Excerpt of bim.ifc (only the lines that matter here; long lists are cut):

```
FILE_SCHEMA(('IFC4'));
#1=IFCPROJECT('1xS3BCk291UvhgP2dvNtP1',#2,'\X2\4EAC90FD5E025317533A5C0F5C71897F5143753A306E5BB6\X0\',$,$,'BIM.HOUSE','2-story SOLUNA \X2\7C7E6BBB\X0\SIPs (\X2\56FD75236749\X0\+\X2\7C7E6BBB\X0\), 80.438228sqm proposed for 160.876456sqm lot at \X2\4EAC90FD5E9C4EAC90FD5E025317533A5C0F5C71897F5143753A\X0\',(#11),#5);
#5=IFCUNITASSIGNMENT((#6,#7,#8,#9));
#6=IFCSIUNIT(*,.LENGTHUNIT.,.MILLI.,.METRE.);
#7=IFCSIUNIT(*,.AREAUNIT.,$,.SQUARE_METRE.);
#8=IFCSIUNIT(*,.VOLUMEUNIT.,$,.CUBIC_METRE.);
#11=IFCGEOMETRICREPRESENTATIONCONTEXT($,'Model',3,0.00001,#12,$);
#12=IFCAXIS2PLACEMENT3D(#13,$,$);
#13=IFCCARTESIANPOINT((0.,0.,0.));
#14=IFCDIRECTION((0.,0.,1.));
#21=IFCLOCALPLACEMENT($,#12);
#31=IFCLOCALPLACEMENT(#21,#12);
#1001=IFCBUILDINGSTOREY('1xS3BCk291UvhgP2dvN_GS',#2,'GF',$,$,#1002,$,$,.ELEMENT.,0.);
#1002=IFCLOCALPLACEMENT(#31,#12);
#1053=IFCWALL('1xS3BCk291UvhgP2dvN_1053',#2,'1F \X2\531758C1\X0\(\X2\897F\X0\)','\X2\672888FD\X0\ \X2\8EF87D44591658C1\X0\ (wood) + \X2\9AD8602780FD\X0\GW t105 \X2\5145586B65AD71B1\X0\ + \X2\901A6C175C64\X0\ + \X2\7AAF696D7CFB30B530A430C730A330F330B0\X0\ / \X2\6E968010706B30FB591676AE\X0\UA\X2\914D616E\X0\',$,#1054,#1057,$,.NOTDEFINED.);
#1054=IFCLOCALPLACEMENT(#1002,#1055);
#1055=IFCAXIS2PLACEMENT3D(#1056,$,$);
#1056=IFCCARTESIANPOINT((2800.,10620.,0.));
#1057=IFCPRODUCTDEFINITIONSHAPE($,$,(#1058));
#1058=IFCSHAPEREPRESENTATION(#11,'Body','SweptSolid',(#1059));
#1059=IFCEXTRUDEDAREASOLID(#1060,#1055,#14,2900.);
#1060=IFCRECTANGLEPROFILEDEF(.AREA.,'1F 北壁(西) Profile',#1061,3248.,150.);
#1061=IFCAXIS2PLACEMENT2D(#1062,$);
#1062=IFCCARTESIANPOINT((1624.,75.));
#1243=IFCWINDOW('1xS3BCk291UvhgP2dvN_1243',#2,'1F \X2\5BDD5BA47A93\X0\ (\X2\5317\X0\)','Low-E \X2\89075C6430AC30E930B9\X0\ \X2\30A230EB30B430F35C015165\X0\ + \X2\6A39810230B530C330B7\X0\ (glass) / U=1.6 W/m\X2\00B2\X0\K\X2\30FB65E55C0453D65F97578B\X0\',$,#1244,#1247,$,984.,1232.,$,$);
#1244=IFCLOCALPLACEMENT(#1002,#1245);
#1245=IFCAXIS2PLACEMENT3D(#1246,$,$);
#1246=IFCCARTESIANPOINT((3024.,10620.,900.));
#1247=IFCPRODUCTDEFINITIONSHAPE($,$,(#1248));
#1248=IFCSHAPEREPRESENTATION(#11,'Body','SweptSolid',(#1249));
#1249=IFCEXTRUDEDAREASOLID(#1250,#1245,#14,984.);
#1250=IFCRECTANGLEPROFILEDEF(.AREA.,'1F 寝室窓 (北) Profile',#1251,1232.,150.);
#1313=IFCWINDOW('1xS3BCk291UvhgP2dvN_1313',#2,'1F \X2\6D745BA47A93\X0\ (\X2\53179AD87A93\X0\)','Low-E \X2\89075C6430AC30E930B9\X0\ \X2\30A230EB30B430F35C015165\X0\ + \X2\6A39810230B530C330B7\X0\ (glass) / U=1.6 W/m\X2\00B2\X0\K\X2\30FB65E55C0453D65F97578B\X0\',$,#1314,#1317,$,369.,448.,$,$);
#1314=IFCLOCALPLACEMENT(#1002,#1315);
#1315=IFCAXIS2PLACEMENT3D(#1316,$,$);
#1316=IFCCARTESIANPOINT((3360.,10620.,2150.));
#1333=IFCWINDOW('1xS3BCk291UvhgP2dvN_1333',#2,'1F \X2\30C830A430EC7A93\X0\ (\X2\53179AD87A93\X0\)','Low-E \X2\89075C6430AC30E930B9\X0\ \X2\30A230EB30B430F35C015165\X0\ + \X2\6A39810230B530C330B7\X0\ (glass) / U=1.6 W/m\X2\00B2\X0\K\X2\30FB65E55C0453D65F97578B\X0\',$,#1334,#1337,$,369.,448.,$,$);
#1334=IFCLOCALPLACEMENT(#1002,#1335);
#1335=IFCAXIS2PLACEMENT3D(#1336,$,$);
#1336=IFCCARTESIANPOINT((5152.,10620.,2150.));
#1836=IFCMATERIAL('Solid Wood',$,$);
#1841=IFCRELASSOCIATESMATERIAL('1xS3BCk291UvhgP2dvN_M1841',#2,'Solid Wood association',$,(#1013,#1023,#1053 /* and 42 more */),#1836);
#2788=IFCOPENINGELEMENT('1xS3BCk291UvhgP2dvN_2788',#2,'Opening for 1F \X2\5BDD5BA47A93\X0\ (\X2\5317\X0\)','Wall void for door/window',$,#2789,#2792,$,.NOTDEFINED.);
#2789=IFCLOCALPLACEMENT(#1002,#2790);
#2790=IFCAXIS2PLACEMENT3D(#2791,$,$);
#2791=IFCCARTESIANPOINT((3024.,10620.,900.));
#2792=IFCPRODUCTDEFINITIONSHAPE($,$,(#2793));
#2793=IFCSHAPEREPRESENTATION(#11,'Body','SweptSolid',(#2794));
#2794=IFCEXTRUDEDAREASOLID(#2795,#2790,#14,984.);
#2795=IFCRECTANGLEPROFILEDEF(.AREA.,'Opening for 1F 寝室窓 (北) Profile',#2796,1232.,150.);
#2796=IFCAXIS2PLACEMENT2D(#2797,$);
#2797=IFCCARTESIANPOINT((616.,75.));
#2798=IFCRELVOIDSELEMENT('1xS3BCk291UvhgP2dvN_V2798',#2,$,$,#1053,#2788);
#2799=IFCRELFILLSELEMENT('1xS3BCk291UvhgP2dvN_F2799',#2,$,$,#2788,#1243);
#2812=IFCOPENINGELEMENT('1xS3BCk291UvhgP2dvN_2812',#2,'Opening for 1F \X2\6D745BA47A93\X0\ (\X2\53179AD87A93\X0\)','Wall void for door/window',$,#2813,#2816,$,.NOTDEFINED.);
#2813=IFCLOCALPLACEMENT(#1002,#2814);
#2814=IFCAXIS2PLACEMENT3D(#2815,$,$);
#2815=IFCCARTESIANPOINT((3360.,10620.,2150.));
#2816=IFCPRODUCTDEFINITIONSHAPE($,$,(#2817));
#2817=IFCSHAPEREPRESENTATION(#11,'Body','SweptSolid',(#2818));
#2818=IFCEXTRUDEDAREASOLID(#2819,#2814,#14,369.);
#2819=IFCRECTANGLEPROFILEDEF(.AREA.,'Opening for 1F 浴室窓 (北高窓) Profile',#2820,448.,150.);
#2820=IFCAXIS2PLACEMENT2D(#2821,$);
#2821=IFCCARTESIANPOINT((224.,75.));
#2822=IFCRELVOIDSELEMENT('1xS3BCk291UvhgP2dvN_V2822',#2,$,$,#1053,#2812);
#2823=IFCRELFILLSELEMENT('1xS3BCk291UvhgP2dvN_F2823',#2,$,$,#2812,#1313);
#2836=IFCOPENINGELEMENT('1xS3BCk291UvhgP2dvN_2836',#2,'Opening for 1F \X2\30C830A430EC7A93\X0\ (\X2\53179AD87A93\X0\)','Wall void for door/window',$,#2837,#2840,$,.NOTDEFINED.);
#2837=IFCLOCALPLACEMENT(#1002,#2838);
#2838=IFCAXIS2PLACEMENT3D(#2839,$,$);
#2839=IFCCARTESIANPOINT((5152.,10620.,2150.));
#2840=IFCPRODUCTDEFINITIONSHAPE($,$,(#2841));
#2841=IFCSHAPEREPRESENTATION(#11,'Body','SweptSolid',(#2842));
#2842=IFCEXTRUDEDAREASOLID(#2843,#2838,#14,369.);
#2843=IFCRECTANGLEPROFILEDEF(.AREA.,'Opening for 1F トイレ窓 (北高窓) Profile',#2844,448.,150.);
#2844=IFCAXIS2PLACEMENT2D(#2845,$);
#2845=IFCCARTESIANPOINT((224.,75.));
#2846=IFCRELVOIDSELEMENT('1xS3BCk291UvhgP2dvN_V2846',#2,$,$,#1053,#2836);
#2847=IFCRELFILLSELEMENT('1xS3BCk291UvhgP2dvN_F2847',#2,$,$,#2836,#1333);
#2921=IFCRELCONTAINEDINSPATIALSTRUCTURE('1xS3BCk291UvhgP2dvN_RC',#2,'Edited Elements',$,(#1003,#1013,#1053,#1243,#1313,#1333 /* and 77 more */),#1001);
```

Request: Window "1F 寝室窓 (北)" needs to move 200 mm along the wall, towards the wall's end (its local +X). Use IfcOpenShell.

```python
import ifcopenshell
import ifcopenshell.api.geometry
import ifcopenshell.util.placement
import ifcopenshell.util.unit

model = ifcopenshell.open("bim.ifc")
unit_scale = ifcopenshell.util.unit.calculate_unit_scale(model)

window = model.by_guid("1xS3BCk291UvhgP2dvN_1243")
opening = window.FillsVoids[0].RelatingOpeningElement
wall = opening.VoidsElements[0].RelatingBuildingElement

wall_matrix = ifcopenshell.util.placement.get_local_placement(wall.ObjectPlacement)
shift = wall_matrix[:3, 0] * 0.2 / unit_scale
before = ifcopenshell.util.placement.get_local_placement(window.ObjectPlacement)[:3, 3].copy()

# The window is not placed relative to its opening, so move both.
for product in (opening, window):
    matrix = ifcopenshell.util.placement.get_local_placement(product.ObjectPlacement)
    matrix[:3, 3] += shift
    ifcopenshell.api.geometry.edit_object_placement(model, product=product, matrix=matrix, is_si=False)

after = ifcopenshell.util.placement.get_local_placement(window.ObjectPlacement)[:3, 3]
print("window moved by", (after - before).round(3) + 0.0)

model.write("bim_v2.ifc")
```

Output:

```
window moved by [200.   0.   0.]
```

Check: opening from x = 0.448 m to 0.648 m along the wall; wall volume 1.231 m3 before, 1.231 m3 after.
